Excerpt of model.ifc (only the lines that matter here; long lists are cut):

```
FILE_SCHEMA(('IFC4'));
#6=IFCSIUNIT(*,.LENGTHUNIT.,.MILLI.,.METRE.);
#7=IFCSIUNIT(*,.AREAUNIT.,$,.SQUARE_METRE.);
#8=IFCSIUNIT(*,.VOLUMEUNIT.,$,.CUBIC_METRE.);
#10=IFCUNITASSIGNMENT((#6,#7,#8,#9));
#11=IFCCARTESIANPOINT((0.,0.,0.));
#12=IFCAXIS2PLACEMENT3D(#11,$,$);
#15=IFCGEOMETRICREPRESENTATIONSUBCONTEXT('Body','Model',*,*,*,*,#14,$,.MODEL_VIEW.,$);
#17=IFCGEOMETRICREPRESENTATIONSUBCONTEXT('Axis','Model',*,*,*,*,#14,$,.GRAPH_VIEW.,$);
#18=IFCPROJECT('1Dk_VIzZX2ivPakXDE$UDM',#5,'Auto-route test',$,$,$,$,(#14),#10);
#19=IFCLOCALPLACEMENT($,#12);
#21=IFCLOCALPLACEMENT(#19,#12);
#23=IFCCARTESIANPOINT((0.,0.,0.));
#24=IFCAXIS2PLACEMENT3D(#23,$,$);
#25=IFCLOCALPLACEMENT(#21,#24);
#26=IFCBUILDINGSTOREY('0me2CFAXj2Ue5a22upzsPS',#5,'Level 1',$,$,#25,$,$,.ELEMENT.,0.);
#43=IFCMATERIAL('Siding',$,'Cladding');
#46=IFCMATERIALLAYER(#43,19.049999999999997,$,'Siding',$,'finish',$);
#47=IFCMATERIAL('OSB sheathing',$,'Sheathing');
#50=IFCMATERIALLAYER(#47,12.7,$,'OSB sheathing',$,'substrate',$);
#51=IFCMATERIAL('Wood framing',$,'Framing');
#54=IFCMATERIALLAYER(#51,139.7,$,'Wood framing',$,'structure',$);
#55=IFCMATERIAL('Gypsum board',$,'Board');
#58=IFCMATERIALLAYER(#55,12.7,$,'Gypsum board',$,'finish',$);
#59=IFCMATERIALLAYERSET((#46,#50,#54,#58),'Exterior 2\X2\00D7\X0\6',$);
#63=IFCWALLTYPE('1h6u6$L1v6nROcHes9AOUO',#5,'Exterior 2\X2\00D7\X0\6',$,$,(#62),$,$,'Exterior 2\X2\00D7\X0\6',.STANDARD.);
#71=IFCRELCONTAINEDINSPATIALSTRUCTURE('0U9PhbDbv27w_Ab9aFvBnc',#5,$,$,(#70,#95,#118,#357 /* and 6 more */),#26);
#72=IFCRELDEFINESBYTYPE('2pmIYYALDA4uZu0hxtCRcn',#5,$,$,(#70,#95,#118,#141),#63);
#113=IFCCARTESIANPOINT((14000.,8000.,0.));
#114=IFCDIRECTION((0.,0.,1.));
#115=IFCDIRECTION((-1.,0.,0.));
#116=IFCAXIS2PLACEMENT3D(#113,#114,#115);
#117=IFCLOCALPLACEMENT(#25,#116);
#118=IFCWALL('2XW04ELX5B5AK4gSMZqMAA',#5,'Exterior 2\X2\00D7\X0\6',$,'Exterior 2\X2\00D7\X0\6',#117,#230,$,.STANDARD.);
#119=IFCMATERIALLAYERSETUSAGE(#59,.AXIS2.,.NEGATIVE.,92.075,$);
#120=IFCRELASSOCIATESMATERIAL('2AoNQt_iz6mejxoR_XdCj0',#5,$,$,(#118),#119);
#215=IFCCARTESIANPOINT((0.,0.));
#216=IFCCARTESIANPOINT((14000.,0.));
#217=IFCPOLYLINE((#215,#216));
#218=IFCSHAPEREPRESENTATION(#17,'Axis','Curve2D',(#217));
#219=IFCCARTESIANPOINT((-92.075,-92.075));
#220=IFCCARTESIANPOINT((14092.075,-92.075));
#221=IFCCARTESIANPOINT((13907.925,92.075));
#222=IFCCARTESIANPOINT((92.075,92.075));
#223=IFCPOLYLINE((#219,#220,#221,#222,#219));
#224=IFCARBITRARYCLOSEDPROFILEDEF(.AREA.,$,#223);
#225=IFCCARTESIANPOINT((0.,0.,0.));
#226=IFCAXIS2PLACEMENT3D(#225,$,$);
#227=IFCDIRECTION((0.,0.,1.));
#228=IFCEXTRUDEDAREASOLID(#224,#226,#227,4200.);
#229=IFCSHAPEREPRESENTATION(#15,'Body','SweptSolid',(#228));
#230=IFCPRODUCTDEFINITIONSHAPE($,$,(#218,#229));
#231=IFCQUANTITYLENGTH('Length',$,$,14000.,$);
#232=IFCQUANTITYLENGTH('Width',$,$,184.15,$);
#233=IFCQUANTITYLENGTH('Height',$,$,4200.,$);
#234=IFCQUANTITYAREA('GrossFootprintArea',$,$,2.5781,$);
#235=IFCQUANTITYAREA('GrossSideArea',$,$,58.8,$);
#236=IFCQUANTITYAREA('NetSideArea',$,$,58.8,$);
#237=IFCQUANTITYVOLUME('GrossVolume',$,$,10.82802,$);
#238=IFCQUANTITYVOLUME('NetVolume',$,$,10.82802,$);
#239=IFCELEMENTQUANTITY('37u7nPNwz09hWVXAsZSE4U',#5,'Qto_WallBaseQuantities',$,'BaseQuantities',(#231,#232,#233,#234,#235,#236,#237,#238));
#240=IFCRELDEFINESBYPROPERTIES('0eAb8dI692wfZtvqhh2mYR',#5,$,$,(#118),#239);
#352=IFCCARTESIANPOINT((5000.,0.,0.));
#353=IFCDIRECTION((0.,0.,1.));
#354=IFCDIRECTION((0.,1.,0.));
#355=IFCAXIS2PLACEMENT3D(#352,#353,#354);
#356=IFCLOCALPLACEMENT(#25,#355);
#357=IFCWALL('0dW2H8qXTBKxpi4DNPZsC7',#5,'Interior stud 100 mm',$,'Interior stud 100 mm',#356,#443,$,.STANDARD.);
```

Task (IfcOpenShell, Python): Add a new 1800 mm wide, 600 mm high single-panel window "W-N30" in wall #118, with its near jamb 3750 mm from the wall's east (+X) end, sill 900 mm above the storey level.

```python
import numpy as np
import ifcopenshell
import ifcopenshell.api.feature
import ifcopenshell.api.geometry
import ifcopenshell.api.pset
import ifcopenshell.api.root
import ifcopenshell.api.spatial
import ifcopenshell.geom
import ifcopenshell.util.element
import ifcopenshell.util.placement
import ifcopenshell.util.representation
import ifcopenshell.util.shape
import ifcopenshell.util.unit

model = ifcopenshell.open("model.ifc")
unit_scale = ifcopenshell.util.unit.calculate_unit_scale(model)
area_scale = ifcopenshell.util.unit.calculate_unit_scale(model, "AREAUNIT")
volume_scale = ifcopenshell.util.unit.calculate_unit_scale(model, "VOLUMEUNIT")
settings = ifcopenshell.geom.settings()


def volume(element):
    """Net volume in cubic metres, openings subtracted."""
    shape = ifcopenshell.geom.create_shape(settings, element)
    return ifcopenshell.util.shape.get_volume(shape.geometry)


wall = model.by_guid("2XW04ELX5B5AK4gSMZqMAA")
storey = ifcopenshell.util.element.get_container(wall, ifc_class="IfcBuildingStorey")
context = ifcopenshell.util.representation.get_context(model, "Model", "Body", "MODEL_VIEW")
before = volume(wall)

width, height, from_end, sill = 1.8, 0.6, 3.75, 0.9  # metres

# The wall runs along its own X axis, and the end named is its -X end.
wall_shape = ifcopenshell.geom.create_shape(settings, wall)
x, y, z = ifcopenshell.util.shape.get_vertices(wall_shape.geometry).T
start = x.min() + from_end
face, thickness = float(y.min()), float(y.max() - y.min())
wall_matrix = ifcopenshell.util.placement.get_local_placement(wall.ObjectPlacement)
level = ifcopenshell.util.placement.get_local_placement(storey.ObjectPlacement)[2, 3]


def in_wall(x, y):
    """Placement at x, y metres in the wall's axes, at sill height."""
    matrix = wall_matrix.copy()
    matrix[:, 3] = wall_matrix @ np.array([x / unit_scale, y / unit_scale, 0.0, 1.0])
    matrix[2, 3] = level + sill / unit_scale
    return matrix


# Opening: a box that overshoots both wall faces by 50 mm.
opening = ifcopenshell.api.root.create_entity(model, ifc_class="IfcOpeningElement", predefined_type="OPENING")
box = ifcopenshell.api.geometry.add_wall_representation(
    model, context=context, length=width, height=height, thickness=thickness + 0.1
)
ifcopenshell.api.geometry.assign_representation(model, product=opening, representation=box)
ifcopenshell.api.geometry.edit_object_placement(model, product=opening, matrix=in_wall(start, face - 0.05), is_si=False)
ifcopenshell.api.feature.add_feature(model, feature=opening, element=wall)

window = ifcopenshell.api.root.create_entity(model, ifc_class="IfcWindow", name="W-N30", predefined_type="WINDOW")
window.OverallWidth, window.OverallHeight = width / unit_scale, height / unit_scale
window.PartitioningType = "SINGLE_PANEL"
body = ifcopenshell.api.geometry.add_window_representation(
    model,
    context=context,
    overall_width=window.OverallWidth,
    overall_height=window.OverallHeight,
    partition_type="SINGLE_PANEL",
)
ifcopenshell.api.geometry.assign_representation(model, product=window, representation=body)
ifcopenshell.api.spatial.assign_container(model, products=[window], relating_structure=storey)
ifcopenshell.api.feature.add_filling(model, opening=opening, element=window)

# Centre the window in the wall's thickness.
ifcopenshell.api.geometry.edit_object_placement(model, product=window, matrix=in_wall(start, face), is_si=False)
window_shape = ifcopenshell.geom.create_shape(settings, window)
depth = ifcopenshell.util.shape.get_vertices(window_shape.geometry)[:, 1]
offset = face + thickness / 2 - (depth.min() + depth.max()) / 2
ifcopenshell.api.geometry.edit_object_placement(model, product=window, matrix=in_wall(start, offset), is_si=False)

after = volume(wall)

# Update the wall's stored quantities.
qto = model.by_id(ifcopenshell.util.element.get_pset(wall, "Qto_WallBaseQuantities", should_inherit=False)["id"])
ifcopenshell.api.pset.edit_qto(model, qto=qto, properties={
    "NetSideArea": after / thickness / area_scale,
    "NetVolume": after / volume_scale,
})

print(f"wall volume {before:.3f} -> {after:.3f} m3")

model.write("model_updated.ifc")
```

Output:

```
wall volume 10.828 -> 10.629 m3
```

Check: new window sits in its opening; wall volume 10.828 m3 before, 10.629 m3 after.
